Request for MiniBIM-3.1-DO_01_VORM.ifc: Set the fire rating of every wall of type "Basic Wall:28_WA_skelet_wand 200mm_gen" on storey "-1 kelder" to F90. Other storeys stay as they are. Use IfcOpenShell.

First a look at what the model holds.

```python
import ifcopenshell
import ifcopenshell.util.element

model = ifcopenshell.open("MiniBIM-3.1-DO_01_VORM.ifc")
print(model.schema)
storey = next(s for s in model.by_type("IfcBuildingStorey") if s.Name == "-1 kelder")
walls = [e for e in ifcopenshell.util.element.get_decomposition(storey) if e.is_a("IfcWall")]
seen = {}
for e in walls:
    element_type = ifcopenshell.util.element.get_type(e)
    key = (element_type.Name if element_type != e and element_type else None, ifcopenshell.util.element.get_pset(e, "Pset_WallCommon", "FireRating"))
    seen[key] = seen.get(key, 0) + 1
for (name, value), count in sorted(seen.items(), key=str):
    print(count, "x", name, "|", value)
```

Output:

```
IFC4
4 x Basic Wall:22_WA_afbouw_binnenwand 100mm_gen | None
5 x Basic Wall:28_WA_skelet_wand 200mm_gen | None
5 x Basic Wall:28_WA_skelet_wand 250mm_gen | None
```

```python
import ifcopenshell
import ifcopenshell.api.pset
import ifcopenshell.util.element

model = ifcopenshell.open("MiniBIM-3.1-DO_01_VORM.ifc")

storey = next(s for s in model.by_type("IfcBuildingStorey") if s.Name == "-1 kelder")
walls = [e for e in ifcopenshell.util.element.get_decomposition(storey) if e.is_a("IfcWall")]

count = 0
for e in walls:
    element_type = ifcopenshell.util.element.get_type(e)
    if element_type in (None, e) or element_type.Name != "Basic Wall:28_WA_skelet_wand 200mm_gen":
        continue
    # add_pset returns the element's existing set when there is one.
    pset = ifcopenshell.api.pset.add_pset(model, product=e, name="Pset_WallCommon")
    ifcopenshell.api.pset.edit_pset(model, pset=pset, properties={"FireRating": "F90"})
    count += 1

print(count, "walls updated")

model.write("MiniBIM-3.1-DO_01_VORM-out.ifc")
```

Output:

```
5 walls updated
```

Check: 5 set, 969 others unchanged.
